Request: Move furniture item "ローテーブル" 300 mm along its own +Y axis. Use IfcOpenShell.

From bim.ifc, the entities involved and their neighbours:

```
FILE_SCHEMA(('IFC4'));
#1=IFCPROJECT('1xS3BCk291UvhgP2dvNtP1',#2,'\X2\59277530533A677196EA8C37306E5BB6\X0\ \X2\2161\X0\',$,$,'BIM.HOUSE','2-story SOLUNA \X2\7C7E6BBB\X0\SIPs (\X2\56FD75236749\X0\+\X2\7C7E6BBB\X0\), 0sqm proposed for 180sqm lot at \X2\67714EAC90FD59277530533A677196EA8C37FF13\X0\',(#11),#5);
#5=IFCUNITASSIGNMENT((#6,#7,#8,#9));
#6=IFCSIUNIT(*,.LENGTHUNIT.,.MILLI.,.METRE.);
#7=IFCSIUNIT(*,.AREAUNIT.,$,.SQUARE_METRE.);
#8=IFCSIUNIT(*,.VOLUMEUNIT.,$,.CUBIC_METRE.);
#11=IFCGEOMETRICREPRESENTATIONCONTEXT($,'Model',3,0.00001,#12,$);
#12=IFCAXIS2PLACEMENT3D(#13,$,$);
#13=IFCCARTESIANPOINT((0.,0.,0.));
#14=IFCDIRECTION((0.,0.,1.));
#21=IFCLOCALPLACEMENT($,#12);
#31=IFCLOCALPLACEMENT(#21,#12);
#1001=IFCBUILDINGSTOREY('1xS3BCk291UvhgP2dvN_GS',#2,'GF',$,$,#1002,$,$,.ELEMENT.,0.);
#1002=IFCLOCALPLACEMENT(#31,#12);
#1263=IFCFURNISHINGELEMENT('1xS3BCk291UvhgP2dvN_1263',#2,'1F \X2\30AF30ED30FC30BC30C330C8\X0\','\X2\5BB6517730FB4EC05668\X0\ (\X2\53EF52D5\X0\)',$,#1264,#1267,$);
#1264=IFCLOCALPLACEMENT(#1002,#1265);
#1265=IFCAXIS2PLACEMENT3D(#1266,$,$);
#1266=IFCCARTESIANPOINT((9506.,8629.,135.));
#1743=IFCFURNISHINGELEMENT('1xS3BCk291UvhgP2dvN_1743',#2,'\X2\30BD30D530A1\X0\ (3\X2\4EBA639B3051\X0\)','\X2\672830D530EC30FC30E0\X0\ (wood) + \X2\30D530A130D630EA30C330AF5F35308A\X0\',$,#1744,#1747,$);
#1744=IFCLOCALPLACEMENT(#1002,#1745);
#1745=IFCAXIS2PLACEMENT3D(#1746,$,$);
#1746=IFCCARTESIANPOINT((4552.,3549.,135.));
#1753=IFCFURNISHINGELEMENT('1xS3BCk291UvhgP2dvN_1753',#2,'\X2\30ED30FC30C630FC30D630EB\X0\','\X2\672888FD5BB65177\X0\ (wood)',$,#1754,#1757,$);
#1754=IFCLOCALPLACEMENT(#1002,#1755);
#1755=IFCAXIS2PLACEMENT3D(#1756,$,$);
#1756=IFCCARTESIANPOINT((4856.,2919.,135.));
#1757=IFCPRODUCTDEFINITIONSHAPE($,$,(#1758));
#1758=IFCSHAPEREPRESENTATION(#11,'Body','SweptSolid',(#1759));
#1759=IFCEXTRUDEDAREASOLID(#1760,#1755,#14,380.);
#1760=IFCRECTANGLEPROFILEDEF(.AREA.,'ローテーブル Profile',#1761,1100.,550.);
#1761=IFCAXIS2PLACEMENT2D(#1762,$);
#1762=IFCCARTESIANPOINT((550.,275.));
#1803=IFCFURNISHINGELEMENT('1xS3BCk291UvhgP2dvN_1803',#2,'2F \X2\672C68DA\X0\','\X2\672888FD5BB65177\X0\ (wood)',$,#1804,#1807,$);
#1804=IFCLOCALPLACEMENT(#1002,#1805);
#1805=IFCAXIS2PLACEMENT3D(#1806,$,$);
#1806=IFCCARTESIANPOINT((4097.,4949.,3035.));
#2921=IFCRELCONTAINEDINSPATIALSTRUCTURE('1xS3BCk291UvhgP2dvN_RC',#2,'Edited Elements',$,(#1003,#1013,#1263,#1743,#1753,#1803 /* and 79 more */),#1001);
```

```python
import ifcopenshell
import ifcopenshell.api.geometry
import ifcopenshell.util.placement
import ifcopenshell.util.unit

model = ifcopenshell.open("bim.ifc")
unit_scale = ifcopenshell.util.unit.calculate_unit_scale(model)

item = model.by_id(1753)
matrix = ifcopenshell.util.placement.get_local_placement(item.ObjectPlacement)
matrix[:3, 3] += matrix[:3, 1] * 0.3 / unit_scale
ifcopenshell.api.geometry.edit_object_placement(model, product=item, matrix=matrix, is_si=False)

print(ifcopenshell.util.placement.get_local_placement(item.ObjectPlacement).round(3) + 0.0)

model.write("bim_edited.ifc")
```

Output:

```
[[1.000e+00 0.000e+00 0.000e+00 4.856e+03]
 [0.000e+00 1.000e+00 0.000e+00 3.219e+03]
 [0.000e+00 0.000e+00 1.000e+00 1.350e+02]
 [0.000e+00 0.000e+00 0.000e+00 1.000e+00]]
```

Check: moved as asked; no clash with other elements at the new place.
